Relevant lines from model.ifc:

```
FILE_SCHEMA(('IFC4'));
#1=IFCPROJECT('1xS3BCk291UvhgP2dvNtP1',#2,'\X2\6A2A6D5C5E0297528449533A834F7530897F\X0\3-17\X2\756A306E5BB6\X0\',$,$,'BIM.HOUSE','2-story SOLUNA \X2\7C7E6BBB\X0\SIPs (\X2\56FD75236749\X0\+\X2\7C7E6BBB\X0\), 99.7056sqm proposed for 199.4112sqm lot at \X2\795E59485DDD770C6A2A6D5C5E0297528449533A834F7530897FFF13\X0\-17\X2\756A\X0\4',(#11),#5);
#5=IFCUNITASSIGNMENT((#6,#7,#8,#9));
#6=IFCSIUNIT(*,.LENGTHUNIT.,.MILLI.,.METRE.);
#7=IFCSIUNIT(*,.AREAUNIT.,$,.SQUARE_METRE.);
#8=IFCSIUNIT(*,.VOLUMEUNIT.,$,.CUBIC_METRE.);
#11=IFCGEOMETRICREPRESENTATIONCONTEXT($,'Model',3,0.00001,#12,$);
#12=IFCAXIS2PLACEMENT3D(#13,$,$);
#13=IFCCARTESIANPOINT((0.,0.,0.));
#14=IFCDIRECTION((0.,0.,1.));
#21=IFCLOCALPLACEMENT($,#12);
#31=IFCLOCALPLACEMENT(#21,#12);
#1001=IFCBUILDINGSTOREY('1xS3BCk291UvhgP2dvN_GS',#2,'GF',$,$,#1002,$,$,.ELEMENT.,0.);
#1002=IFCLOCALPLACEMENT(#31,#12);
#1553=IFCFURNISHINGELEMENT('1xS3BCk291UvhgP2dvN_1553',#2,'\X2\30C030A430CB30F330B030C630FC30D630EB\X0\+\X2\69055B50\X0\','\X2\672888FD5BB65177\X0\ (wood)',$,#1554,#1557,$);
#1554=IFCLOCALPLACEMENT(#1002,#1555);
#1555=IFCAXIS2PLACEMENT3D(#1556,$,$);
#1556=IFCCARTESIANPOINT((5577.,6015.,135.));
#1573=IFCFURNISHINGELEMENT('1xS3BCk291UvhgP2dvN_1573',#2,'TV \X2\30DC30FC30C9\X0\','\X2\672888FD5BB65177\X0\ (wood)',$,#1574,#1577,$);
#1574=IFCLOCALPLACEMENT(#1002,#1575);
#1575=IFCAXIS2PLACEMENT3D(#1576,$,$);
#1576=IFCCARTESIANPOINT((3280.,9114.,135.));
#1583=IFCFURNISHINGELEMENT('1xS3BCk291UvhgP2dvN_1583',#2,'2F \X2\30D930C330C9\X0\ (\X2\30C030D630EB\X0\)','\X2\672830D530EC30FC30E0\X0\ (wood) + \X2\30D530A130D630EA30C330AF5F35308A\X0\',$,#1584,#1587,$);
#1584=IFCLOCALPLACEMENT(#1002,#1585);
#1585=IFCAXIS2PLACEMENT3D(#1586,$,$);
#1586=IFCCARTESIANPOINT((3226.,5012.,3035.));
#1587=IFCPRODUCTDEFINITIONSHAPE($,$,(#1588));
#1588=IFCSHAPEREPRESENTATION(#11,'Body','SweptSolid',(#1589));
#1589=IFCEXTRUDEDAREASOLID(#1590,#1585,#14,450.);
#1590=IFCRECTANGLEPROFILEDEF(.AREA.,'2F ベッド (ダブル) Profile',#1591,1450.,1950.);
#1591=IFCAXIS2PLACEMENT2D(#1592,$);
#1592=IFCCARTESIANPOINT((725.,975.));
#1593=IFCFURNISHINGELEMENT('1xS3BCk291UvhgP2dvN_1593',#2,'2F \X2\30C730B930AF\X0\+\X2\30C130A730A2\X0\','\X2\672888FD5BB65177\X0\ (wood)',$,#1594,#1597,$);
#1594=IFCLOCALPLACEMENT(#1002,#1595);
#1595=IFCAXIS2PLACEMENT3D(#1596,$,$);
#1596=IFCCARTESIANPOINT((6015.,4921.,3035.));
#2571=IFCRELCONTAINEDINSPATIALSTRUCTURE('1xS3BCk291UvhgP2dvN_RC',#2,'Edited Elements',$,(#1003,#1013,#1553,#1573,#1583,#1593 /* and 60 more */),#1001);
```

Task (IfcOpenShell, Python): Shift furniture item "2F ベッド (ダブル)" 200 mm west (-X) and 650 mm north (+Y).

```python
import ifcopenshell
import ifcopenshell.api.geometry
import ifcopenshell.util.placement

model = ifcopenshell.open("model.ifc")

item = model.by_id(1583)
matrix = ifcopenshell.util.placement.get_local_placement(item.ObjectPlacement)
matrix[0, 3] -= 200.0
matrix[1, 3] += 650.0
ifcopenshell.api.geometry.edit_object_placement(model, product=item, matrix=matrix, is_si=False)

print(ifcopenshell.util.placement.get_local_placement(item.ObjectPlacement).round(3) + 0.0)

model.write("model_rev.ifc")
```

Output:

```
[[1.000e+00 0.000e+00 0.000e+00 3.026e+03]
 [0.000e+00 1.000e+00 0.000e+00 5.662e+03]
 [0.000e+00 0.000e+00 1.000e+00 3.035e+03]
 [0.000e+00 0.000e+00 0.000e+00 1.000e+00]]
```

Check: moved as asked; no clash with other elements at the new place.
